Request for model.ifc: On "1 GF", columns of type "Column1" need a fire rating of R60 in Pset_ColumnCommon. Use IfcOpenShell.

First a look at what the model holds.

```python
import ifcopenshell
import ifcopenshell.util.element

model = ifcopenshell.open("model.ifc")
print(model.schema)
storey = next(s for s in model.by_type("IfcBuildingStorey") if s.Name == "1 GF")
columns = [e for e in ifcopenshell.util.element.get_decomposition(storey) if e.is_a("IfcColumn")]
seen = {}
for e in columns:
    element_type = ifcopenshell.util.element.get_type(e)
    key = (element_type.Name if element_type != e and element_type else None, ifcopenshell.util.element.get_pset(e, "Pset_ColumnCommon", "FireRating"))
    seen[key] = seen.get(key, 0) + 1
for (name, value), count in sorted(seen.items(), key=str):
    print(count, "x", name, "|", value)
```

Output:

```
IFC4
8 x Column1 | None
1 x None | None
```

```python
import ifcopenshell
import ifcopenshell.api.pset
import ifcopenshell.util.element

model = ifcopenshell.open("model.ifc")

storey = next(s for s in model.by_type("IfcBuildingStorey") if s.Name == "1 GF")
columns = [e for e in ifcopenshell.util.element.get_decomposition(storey) if e.is_a("IfcColumn")]

count = 0
for e in columns:
    element_type = ifcopenshell.util.element.get_type(e)
    if element_type in (None, e) or element_type.Name != "Column1":
        continue
    # add_pset returns the element's existing set when there is one.
    pset = ifcopenshell.api.pset.add_pset(model, product=e, name="Pset_ColumnCommon")
    ifcopenshell.api.pset.edit_pset(model, pset=pset, properties={"FireRating": "R60"})
    count += 1

print(count, "columns updated")

model.write("model-out.ifc")
```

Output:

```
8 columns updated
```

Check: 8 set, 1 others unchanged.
